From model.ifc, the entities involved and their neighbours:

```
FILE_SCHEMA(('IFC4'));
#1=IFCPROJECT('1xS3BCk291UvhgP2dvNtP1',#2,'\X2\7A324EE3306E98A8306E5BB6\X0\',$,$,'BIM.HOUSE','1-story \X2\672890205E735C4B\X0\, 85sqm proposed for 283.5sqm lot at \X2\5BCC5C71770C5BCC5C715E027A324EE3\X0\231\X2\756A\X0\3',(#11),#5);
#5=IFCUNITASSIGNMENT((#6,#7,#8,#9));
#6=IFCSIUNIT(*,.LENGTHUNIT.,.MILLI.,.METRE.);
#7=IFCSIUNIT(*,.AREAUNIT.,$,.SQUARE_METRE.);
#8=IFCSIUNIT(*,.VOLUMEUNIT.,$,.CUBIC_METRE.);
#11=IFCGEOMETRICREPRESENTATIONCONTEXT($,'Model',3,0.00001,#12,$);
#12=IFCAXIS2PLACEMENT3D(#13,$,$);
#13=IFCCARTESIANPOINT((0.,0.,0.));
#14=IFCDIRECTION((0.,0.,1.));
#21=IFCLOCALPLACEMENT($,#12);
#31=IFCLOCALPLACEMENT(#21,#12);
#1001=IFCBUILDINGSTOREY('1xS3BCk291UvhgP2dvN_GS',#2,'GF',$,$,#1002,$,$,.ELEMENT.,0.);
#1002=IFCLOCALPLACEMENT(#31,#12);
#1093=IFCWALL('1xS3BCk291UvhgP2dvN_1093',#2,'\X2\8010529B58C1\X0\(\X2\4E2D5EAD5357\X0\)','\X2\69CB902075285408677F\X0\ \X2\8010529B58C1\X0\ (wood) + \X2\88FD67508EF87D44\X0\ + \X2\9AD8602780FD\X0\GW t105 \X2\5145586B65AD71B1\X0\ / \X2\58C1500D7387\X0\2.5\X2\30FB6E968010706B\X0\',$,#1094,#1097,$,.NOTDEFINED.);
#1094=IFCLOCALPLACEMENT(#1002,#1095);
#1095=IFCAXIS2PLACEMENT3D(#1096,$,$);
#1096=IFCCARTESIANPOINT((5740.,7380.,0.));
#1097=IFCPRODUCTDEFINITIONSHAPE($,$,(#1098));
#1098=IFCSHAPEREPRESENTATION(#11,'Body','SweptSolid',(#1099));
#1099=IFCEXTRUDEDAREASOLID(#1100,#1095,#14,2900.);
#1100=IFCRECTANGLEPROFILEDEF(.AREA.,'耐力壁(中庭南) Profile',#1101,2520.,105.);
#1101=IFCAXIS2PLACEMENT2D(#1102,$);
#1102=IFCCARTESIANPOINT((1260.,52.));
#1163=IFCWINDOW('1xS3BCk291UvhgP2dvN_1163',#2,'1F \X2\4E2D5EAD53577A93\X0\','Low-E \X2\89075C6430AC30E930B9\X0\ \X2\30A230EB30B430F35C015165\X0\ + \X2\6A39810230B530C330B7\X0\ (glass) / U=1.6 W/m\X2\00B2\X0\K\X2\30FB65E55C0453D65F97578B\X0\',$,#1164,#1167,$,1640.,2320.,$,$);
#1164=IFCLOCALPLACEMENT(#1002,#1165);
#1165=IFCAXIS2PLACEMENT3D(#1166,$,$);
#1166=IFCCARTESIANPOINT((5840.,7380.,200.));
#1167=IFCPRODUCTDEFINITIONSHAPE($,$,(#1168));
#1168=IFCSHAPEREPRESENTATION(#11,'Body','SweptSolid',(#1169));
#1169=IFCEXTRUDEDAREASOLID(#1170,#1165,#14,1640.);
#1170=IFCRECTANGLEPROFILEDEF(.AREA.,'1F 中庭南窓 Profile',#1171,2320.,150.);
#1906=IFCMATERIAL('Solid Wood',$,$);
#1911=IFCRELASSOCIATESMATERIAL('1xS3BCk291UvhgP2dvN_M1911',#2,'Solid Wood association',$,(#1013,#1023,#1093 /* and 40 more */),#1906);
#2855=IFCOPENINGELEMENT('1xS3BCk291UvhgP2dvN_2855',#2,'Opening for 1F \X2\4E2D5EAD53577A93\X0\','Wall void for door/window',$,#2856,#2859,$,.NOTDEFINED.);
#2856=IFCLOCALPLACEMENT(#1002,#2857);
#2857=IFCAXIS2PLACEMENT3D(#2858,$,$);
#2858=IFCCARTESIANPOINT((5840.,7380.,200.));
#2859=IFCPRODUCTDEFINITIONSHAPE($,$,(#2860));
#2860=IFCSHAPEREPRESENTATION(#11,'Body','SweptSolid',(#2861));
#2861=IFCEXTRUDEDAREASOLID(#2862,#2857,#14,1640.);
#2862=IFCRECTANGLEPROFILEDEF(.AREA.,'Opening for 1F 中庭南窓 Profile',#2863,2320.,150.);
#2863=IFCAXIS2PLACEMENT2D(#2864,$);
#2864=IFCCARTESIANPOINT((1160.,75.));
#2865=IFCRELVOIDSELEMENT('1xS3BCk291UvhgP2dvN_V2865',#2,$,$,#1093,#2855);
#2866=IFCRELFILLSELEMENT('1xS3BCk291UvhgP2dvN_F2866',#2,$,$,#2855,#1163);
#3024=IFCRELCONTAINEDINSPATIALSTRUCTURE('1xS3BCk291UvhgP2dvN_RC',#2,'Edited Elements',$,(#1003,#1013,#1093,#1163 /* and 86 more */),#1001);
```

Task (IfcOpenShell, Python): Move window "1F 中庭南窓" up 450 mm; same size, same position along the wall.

```python
import numpy as np
import ifcopenshell
import ifcopenshell.api.geometry
import ifcopenshell.util.placement
import ifcopenshell.util.unit

model = ifcopenshell.open("model.ifc")
unit_scale = ifcopenshell.util.unit.calculate_unit_scale(model)

window = model.by_guid("1xS3BCk291UvhgP2dvN_1163")
opening = window.FillsVoids[0].RelatingOpeningElement
dz = 450.0

shift = np.array([0.0, 0.0, dz])
# The window is not placed relative to its opening, so move both.
for product in (opening, window):
    matrix = ifcopenshell.util.placement.get_local_placement(product.ObjectPlacement)
    matrix[:3, 3] += shift
    ifcopenshell.api.geometry.edit_object_placement(model, product=product, matrix=matrix, is_si=False)

print(f"moved by {dz * unit_scale:+.3f} m")

model.write("model_edited.ifc")
```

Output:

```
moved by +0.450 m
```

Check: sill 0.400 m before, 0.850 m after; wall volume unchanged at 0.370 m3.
